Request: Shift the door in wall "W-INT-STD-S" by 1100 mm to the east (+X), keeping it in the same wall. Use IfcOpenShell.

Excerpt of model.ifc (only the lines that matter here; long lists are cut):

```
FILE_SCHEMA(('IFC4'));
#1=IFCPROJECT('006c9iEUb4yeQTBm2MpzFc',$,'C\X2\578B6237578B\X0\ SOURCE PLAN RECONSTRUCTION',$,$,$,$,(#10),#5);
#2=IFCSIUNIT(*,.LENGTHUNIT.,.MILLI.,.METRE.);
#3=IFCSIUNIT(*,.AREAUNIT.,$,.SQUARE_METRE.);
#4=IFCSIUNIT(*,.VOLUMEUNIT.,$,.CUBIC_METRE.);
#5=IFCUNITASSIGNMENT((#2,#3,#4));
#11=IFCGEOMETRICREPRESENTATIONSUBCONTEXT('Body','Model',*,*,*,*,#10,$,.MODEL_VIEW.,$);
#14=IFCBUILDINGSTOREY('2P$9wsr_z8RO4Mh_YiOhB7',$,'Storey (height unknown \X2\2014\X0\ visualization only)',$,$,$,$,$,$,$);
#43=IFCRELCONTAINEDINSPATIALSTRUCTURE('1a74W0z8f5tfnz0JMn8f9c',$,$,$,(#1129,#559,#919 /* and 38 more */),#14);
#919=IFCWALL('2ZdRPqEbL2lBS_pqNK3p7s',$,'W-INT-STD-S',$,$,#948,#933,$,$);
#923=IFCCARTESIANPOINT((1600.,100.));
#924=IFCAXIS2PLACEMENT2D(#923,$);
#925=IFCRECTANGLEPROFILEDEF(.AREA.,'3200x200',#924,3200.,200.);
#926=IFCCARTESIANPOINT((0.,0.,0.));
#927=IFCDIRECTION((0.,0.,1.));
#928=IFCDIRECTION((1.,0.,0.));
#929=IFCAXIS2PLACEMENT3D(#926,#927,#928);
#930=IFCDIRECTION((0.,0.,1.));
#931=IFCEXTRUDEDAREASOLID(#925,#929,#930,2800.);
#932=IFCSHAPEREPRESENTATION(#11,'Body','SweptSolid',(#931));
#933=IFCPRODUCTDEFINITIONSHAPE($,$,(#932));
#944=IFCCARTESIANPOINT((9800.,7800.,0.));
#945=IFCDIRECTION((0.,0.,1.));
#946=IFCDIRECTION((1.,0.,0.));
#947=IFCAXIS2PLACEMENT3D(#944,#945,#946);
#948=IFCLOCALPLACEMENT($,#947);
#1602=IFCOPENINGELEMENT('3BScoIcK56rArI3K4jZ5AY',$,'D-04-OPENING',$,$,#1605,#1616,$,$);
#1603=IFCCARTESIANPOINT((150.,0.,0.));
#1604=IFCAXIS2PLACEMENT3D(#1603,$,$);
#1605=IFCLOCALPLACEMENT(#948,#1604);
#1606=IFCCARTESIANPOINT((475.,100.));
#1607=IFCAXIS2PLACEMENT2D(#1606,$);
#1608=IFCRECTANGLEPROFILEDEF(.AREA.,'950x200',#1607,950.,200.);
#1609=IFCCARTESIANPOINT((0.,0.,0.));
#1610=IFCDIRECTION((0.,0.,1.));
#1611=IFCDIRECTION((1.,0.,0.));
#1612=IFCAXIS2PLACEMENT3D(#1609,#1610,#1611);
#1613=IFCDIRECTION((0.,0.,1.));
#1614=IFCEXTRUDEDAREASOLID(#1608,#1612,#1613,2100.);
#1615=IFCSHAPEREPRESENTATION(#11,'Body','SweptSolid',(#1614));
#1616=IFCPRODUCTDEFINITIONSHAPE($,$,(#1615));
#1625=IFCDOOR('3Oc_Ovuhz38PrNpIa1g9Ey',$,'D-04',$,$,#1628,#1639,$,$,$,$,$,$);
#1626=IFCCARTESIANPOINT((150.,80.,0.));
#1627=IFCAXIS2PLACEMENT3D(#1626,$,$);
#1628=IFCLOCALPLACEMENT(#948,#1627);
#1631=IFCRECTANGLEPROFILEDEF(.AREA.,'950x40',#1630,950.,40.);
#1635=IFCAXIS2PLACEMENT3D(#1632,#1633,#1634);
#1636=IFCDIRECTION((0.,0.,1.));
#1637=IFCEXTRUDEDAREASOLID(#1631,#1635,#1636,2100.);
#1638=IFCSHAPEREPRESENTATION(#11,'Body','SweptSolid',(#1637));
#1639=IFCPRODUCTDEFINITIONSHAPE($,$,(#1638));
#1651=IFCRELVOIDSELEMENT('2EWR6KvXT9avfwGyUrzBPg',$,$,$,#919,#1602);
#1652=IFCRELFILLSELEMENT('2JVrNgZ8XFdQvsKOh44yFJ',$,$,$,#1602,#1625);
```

```python
import ifcopenshell
import ifcopenshell.api.geometry
import ifcopenshell.util.placement

model = ifcopenshell.open("model.ifc")

door = model.by_guid("3Oc_Ovuhz38PrNpIa1g9Ey")
opening = door.FillsVoids[0].RelatingOpeningElement
wall = opening.VoidsElements[0].RelatingBuildingElement

wall_matrix = ifcopenshell.util.placement.get_local_placement(wall.ObjectPlacement)
shift = wall_matrix[:3, 0] * 1100.0
before = ifcopenshell.util.placement.get_local_placement(door.ObjectPlacement)[:3, 3].copy()

# The door is not placed relative to its opening, so move both.
for product in (opening, door):
    matrix = ifcopenshell.util.placement.get_local_placement(product.ObjectPlacement)
    matrix[:3, 3] += shift
    ifcopenshell.api.geometry.edit_object_placement(model, product=product, matrix=matrix, is_si=False)

after = ifcopenshell.util.placement.get_local_placement(door.ObjectPlacement)[:3, 3]
print("door moved by", (after - before).round(3) + 0.0)

model.write("model_v2.ifc")
```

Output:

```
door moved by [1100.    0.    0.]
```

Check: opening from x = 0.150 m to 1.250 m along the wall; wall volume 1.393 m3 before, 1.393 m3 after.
